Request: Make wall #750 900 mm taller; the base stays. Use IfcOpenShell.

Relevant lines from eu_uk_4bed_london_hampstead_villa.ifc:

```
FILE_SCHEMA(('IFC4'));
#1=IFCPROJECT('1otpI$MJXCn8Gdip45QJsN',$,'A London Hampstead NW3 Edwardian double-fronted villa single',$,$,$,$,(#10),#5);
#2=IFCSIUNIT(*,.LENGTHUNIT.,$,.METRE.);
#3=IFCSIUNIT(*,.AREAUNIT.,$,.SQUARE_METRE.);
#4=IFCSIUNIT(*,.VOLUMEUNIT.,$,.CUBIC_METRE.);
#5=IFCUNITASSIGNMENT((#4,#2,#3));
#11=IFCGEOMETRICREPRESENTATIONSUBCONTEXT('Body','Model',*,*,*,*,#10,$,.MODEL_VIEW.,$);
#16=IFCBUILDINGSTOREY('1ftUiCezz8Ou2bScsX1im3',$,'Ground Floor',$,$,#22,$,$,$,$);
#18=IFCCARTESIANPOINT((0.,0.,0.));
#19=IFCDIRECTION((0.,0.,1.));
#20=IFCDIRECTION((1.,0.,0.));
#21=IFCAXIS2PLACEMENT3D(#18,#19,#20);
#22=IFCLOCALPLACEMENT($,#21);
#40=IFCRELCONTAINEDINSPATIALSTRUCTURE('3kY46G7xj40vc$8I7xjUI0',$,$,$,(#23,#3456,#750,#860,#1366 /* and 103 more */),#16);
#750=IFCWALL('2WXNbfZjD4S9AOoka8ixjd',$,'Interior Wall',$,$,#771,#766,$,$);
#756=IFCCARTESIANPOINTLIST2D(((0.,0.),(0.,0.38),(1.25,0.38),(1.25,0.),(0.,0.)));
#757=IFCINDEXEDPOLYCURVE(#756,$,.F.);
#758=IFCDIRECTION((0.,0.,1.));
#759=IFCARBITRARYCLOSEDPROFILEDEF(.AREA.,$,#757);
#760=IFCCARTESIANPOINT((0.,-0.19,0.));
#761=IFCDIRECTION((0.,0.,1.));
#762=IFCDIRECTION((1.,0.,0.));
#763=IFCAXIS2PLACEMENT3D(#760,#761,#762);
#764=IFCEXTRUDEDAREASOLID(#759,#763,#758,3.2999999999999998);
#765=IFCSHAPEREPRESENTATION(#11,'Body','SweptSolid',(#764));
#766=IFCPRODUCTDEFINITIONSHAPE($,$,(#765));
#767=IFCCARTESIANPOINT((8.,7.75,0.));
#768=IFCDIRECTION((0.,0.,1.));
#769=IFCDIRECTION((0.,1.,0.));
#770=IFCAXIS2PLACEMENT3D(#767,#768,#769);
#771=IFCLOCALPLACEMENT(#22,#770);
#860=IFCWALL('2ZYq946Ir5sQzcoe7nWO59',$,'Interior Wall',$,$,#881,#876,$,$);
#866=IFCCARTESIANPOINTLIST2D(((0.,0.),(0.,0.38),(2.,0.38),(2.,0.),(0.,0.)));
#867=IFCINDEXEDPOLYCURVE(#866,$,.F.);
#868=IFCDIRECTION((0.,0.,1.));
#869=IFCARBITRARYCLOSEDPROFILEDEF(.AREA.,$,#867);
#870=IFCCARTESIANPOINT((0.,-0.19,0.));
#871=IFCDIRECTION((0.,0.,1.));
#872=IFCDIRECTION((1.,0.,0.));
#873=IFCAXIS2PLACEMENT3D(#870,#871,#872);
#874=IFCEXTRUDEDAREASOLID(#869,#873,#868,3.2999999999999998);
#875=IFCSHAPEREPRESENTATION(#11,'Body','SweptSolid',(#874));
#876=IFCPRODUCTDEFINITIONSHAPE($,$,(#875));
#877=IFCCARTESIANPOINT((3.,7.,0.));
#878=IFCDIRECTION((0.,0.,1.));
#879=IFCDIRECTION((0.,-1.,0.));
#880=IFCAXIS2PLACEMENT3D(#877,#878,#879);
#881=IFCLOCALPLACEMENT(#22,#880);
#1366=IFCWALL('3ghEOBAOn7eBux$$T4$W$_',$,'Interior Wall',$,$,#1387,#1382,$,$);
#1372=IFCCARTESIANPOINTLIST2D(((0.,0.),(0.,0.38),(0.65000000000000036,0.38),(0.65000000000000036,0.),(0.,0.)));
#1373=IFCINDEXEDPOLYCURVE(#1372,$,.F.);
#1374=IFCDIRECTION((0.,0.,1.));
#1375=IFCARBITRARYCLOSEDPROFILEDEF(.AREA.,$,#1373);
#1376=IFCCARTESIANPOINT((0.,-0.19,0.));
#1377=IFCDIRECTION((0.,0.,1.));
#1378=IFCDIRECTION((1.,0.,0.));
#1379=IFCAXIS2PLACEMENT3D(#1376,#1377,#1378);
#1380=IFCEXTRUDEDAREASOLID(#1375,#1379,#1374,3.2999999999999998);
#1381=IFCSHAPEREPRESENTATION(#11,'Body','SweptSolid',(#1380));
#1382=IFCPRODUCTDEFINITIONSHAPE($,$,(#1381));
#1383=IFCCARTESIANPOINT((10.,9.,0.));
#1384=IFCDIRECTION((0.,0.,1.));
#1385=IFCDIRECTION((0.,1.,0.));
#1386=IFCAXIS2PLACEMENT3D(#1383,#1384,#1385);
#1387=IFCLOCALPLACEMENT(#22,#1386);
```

```python
import ifcopenshell
import ifcopenshell.geom
import ifcopenshell.util.representation
import ifcopenshell.util.shape
import ifcopenshell.util.unit

model = ifcopenshell.open("eu_uk_4bed_london_hampstead_villa.ifc")
unit_scale = ifcopenshell.util.unit.calculate_unit_scale(model)
settings = ifcopenshell.geom.settings()


def volume(element):
    """Net volume in cubic metres, openings subtracted."""
    shape = ifcopenshell.geom.create_shape(settings, element)
    return ifcopenshell.util.shape.get_volume(shape.geometry)


wall = model.by_id(750)
before = volume(wall)

body = ifcopenshell.util.representation.get_representation(wall, "Model", "Body")
solid = body.Items[0]
old_height = solid.Depth
solid.Depth += 0.9 / unit_scale
after = volume(wall)

print(f"height {old_height:g} -> {solid.Depth:g}, volume {before:.3f} -> {after:.3f} m3")

model.write("eu_uk_4bed_london_hampstead_villa_rev.ifc")
```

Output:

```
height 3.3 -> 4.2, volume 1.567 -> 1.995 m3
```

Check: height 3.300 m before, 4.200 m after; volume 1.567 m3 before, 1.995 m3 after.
